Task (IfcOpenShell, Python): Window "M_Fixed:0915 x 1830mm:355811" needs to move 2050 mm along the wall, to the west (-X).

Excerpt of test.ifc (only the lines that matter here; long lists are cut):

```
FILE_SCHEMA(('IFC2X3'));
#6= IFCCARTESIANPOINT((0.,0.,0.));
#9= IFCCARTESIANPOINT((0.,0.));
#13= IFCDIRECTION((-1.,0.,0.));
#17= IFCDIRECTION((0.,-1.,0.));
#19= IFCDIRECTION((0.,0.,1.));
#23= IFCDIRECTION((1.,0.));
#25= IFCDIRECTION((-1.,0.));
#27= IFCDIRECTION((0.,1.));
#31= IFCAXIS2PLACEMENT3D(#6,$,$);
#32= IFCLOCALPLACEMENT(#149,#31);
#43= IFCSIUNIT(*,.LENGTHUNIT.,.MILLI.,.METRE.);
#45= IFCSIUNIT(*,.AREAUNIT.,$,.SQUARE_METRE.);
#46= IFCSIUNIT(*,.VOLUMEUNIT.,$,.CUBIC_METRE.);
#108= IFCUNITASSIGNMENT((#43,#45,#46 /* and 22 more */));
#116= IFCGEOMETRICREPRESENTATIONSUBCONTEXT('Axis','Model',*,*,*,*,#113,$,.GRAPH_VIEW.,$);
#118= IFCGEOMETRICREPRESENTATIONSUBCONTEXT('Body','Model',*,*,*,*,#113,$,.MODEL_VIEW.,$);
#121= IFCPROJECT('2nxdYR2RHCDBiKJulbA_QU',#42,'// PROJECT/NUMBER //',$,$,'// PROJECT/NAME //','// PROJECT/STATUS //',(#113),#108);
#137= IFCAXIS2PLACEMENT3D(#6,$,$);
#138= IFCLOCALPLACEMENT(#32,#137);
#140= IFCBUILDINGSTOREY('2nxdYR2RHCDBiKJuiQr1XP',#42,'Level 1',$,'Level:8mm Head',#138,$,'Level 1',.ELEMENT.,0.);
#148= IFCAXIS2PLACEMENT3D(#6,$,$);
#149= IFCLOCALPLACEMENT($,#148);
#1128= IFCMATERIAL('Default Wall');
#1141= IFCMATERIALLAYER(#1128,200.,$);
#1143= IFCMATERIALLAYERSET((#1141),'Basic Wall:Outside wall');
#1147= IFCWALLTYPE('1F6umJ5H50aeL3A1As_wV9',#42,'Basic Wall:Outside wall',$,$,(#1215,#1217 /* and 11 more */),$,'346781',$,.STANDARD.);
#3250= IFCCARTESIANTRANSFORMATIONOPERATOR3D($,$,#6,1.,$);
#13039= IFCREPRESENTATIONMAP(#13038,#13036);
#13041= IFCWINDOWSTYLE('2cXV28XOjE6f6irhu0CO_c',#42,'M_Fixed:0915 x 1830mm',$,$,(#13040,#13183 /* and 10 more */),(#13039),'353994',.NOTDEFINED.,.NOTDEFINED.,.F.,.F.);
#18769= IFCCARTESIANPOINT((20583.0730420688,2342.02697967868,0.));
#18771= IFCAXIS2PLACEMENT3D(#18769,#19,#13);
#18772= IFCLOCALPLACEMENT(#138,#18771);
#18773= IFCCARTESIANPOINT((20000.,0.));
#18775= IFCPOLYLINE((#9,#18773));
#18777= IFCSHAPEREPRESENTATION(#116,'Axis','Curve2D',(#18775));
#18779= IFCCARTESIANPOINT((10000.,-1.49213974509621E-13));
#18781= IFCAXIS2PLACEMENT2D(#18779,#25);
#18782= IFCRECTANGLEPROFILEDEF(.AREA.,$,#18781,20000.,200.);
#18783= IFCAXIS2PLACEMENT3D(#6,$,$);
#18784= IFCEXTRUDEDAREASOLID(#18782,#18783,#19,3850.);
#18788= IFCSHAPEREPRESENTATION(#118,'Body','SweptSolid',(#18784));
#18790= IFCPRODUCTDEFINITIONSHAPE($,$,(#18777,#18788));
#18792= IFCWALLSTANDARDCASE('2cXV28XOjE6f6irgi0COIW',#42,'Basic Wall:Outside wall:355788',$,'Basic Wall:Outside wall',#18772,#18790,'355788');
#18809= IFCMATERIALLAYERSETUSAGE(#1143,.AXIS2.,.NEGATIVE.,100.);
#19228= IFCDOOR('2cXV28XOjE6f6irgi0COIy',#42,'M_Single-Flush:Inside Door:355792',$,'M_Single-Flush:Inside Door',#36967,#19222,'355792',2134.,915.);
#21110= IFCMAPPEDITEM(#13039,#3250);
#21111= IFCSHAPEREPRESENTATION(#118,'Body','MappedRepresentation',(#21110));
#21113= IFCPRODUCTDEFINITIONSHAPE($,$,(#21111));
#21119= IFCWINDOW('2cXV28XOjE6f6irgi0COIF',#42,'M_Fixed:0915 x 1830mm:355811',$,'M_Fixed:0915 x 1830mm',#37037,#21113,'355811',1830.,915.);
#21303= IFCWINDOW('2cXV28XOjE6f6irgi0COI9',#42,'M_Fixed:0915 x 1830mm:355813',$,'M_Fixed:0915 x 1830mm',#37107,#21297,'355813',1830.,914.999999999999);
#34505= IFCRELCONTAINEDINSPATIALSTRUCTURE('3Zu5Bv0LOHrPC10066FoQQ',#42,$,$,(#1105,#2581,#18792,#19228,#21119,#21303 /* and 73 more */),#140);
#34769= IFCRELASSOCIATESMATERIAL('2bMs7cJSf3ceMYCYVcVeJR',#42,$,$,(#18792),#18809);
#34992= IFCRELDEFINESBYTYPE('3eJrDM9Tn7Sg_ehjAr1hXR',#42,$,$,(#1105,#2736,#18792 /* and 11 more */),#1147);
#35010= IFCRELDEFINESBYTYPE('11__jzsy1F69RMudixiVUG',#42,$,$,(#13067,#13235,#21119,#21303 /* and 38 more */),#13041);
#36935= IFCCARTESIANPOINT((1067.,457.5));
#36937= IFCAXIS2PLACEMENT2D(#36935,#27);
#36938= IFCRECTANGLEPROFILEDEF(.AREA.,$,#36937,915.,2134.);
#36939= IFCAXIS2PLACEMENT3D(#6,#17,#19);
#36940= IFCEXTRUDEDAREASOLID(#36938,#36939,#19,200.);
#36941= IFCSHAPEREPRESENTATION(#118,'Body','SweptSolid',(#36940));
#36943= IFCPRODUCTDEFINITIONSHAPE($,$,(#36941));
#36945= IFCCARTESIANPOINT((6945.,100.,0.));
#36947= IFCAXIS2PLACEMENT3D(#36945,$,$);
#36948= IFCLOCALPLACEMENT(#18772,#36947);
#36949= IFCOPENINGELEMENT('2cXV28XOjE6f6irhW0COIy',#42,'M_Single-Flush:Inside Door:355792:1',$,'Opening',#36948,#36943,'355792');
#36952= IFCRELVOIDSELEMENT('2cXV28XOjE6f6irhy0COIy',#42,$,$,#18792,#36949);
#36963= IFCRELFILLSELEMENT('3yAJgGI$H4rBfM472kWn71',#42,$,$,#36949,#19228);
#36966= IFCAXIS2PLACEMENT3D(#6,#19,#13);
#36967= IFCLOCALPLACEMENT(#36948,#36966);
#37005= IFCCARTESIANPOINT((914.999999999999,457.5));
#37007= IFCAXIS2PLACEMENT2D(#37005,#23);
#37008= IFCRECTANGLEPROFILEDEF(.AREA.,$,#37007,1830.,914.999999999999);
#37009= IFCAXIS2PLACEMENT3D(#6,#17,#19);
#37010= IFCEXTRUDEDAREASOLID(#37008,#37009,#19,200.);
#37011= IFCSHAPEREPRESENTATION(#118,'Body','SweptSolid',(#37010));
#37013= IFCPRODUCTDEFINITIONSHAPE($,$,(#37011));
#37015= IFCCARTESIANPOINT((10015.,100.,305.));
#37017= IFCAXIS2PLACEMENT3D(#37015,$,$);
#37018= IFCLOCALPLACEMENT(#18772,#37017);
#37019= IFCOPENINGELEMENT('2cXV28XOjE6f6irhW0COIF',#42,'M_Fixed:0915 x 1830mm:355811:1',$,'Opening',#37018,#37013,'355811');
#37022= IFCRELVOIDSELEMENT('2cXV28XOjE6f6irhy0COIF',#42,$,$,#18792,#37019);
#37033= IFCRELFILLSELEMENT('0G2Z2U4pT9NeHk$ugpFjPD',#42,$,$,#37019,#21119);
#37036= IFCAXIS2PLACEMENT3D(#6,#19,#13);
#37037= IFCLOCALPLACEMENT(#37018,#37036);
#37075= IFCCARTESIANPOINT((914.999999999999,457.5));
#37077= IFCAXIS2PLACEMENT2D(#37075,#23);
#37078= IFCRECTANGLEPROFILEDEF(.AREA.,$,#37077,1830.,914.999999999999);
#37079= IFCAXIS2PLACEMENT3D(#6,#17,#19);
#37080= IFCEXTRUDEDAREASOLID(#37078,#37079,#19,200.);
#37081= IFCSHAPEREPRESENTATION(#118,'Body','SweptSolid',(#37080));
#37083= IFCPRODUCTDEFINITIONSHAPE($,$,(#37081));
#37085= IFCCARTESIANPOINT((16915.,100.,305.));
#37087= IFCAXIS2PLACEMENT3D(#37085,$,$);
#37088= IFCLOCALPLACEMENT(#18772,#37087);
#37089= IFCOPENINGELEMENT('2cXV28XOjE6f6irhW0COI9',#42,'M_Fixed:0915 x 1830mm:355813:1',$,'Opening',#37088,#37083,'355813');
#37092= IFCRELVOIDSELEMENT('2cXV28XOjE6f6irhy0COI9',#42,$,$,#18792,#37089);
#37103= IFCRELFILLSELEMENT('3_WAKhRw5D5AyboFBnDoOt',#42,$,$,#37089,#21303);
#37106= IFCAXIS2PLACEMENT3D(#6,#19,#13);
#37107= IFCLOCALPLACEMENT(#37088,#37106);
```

```python
import ifcopenshell
import ifcopenshell.api.geometry
import ifcopenshell.util.placement

model = ifcopenshell.open("test.ifc")

window = model.by_id(21119)
opening = window.FillsVoids[0].RelatingOpeningElement
wall = opening.VoidsElements[0].RelatingBuildingElement

wall_matrix = ifcopenshell.util.placement.get_local_placement(wall.ObjectPlacement)
shift = wall_matrix[:3, 0] * 2050.0
before = ifcopenshell.util.placement.get_local_placement(window.ObjectPlacement)[:3, 3].copy()

# The window is placed relative to its opening, so it follows when the opening moves.
matrix = ifcopenshell.util.placement.get_local_placement(opening.ObjectPlacement)
matrix[:3, 3] += shift
ifcopenshell.api.geometry.edit_object_placement(
    model, product=opening, matrix=matrix, is_si=False, should_transform_children=True
)

after = ifcopenshell.util.placement.get_local_placement(window.ObjectPlacement)[:3, 3]
print("window moved by", (after - before).round(3) + 0.0)

model.write("test_rev.ifc")
```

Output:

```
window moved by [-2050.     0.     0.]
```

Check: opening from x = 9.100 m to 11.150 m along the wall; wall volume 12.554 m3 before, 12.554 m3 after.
